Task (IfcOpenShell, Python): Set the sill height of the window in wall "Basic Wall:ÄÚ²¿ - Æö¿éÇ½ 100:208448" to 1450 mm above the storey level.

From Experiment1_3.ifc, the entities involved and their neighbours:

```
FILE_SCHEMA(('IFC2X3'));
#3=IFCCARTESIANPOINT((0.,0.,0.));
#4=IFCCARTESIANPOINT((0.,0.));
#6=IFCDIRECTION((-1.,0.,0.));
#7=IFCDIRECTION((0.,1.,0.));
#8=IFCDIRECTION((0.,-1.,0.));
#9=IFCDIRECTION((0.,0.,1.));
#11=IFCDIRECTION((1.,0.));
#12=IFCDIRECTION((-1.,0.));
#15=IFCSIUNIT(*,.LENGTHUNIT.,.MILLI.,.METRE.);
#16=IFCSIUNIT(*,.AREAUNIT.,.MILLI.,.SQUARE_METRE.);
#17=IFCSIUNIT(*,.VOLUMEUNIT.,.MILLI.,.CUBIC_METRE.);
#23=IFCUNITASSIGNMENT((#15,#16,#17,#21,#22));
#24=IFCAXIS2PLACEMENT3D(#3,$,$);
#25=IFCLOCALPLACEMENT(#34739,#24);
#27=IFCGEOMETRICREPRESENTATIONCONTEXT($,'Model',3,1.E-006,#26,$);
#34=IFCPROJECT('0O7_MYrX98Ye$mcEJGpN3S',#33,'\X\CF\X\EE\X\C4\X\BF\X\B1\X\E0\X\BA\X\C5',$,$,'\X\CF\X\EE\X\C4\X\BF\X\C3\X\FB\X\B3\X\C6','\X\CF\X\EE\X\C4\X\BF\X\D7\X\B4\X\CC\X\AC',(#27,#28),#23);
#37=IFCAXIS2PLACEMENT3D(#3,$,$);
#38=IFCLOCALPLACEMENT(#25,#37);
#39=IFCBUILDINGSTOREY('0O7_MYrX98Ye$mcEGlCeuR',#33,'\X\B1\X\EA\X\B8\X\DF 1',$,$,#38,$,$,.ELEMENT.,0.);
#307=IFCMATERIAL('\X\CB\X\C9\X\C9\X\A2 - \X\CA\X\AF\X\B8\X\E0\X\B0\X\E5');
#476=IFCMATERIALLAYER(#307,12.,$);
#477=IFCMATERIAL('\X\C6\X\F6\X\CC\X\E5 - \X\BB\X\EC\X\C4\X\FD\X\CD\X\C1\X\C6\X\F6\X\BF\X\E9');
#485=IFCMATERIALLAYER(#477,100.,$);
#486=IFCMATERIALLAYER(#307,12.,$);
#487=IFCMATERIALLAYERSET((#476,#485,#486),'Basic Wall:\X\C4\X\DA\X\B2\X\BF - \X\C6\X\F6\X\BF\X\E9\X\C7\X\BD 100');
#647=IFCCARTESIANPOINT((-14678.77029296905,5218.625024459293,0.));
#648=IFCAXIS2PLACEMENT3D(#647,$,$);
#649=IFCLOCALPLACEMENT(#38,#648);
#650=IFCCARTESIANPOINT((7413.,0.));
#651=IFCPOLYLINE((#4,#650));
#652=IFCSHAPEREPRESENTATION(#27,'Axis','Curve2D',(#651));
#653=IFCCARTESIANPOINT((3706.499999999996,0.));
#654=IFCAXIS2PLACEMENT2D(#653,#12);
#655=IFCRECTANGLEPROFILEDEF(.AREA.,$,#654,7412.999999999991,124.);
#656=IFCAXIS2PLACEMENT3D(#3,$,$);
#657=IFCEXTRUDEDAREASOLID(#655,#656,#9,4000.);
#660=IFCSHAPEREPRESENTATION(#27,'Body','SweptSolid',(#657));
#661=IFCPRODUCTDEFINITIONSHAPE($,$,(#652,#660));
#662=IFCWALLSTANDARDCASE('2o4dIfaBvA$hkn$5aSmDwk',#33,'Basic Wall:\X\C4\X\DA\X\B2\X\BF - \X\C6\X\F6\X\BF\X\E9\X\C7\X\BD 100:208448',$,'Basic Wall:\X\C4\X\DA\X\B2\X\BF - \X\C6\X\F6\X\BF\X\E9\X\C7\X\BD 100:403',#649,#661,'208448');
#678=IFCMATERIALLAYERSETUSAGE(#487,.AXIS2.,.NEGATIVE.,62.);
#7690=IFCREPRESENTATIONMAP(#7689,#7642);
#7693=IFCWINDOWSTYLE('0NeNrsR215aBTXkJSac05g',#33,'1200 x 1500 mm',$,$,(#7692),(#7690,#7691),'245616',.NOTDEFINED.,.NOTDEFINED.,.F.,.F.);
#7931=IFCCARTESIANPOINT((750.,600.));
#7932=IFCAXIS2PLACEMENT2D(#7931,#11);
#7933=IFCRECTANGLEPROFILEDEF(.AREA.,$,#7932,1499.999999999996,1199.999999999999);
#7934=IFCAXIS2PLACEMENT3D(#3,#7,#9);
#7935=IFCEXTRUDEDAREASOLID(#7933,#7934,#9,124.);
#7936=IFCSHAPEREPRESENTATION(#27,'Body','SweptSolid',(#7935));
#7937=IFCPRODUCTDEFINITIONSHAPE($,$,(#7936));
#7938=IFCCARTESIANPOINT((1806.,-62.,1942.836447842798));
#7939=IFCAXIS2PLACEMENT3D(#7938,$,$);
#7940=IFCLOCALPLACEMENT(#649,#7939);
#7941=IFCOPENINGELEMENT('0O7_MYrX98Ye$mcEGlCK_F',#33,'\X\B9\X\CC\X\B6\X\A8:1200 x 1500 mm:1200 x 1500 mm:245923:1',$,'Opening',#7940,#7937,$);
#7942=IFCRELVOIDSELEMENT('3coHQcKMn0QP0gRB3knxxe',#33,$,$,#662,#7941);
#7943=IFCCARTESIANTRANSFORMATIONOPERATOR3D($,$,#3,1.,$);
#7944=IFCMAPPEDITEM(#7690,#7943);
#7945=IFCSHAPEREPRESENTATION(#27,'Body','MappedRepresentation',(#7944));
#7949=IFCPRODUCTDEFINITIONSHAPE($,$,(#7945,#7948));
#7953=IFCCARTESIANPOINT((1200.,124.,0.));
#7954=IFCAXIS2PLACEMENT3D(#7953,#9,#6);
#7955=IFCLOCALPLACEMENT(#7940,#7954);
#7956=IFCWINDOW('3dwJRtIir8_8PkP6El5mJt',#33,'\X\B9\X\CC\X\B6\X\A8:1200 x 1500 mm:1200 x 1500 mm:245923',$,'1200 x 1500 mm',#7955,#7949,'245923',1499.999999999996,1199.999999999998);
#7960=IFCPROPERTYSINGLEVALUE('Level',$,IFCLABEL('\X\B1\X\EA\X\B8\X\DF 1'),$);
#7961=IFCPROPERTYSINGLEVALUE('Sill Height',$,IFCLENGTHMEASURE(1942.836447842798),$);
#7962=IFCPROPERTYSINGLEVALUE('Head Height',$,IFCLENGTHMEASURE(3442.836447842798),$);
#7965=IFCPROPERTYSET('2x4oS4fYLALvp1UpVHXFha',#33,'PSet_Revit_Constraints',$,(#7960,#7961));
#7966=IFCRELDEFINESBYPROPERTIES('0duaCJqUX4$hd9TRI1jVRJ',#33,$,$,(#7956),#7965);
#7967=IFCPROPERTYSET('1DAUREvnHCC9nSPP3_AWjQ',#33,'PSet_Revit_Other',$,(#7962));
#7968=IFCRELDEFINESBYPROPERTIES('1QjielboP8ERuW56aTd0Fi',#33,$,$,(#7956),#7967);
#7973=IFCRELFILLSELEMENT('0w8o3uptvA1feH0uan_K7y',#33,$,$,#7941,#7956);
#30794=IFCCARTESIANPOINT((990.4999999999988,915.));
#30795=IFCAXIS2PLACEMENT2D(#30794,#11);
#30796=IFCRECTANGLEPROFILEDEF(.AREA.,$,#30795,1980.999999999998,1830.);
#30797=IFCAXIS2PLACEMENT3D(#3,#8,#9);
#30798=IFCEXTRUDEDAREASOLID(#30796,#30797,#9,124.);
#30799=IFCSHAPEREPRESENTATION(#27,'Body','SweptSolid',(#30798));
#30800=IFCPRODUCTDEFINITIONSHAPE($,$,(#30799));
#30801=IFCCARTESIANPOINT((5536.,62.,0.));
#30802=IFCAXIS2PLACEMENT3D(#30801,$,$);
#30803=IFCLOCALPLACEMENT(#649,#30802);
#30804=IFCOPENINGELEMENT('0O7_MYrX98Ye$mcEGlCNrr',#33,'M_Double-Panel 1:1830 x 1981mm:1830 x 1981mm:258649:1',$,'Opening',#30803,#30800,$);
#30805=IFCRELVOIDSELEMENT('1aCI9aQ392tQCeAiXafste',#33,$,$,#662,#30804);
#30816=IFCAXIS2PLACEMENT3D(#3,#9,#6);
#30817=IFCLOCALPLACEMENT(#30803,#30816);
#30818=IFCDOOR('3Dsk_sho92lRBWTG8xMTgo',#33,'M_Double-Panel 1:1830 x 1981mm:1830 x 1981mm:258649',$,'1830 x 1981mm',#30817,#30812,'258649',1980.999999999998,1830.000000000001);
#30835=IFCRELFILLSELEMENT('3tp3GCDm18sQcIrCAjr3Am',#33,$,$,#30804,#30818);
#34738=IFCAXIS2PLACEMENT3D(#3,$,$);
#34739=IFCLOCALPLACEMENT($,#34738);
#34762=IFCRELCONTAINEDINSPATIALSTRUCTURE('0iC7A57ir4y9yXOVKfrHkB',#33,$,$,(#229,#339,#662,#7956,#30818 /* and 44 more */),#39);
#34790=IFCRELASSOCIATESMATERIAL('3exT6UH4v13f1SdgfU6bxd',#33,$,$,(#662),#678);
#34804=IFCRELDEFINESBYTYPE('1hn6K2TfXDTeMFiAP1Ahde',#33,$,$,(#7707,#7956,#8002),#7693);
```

```python
import numpy as np
import ifcopenshell
import ifcopenshell.api.geometry
import ifcopenshell.api.pset
import ifcopenshell.geom
import ifcopenshell.util.element
import ifcopenshell.util.placement
import ifcopenshell.util.shape
import ifcopenshell.util.unit

model = ifcopenshell.open("Experiment1_3.ifc")
unit_scale = ifcopenshell.util.unit.calculate_unit_scale(model)

window = model.by_guid("3dwJRtIir8_8PkP6El5mJt")
opening = window.FillsVoids[0].RelatingOpeningElement
storey = ifcopenshell.util.element.get_container(window, ifc_class="IfcBuildingStorey")
level = ifcopenshell.util.placement.get_local_placement(storey.ObjectPlacement)[2, 3]

# The opening's origin need not be at the sill, so measure its lowest point.
shape = ifcopenshell.geom.create_shape(ifcopenshell.geom.settings(), opening)
bottom = ifcopenshell.util.shape.get_shape_bottom_elevation(shape, shape.geometry) / unit_scale
dz = level + 1.45 / unit_scale - bottom

shift = np.array([0.0, 0.0, dz])
# The window is placed relative to its opening, so it follows when the opening moves.
matrix = ifcopenshell.util.placement.get_local_placement(opening.ObjectPlacement)
matrix[:3, 3] += shift
ifcopenshell.api.geometry.edit_object_placement(
    model, product=opening, matrix=matrix, is_si=False, should_transform_children=True
)

# Keep the stored heights in step.
pset = model.by_id(ifcopenshell.util.element.get_pset(window, "PSet_Revit_Constraints", should_inherit=False)["id"])
ifcopenshell.api.pset.edit_pset(model, pset=pset, properties={
    "Sill Height": model.create_entity("IfcLengthMeasure", ifcopenshell.util.element.get_pset(window, "PSet_Revit_Constraints", "Sill Height") + dz),
})
pset = model.by_id(ifcopenshell.util.element.get_pset(window, "PSet_Revit_Other", should_inherit=False)["id"])
ifcopenshell.api.pset.edit_pset(model, pset=pset, properties={
    "Head Height": model.create_entity("IfcLengthMeasure", ifcopenshell.util.element.get_pset(window, "PSet_Revit_Other", "Head Height") + dz),
})

print(f"moved by {dz * unit_scale:+.3f} m")

model.write("Experiment1_3_updated.ifc")
```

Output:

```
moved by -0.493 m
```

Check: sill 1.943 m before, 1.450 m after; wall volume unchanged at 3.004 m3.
